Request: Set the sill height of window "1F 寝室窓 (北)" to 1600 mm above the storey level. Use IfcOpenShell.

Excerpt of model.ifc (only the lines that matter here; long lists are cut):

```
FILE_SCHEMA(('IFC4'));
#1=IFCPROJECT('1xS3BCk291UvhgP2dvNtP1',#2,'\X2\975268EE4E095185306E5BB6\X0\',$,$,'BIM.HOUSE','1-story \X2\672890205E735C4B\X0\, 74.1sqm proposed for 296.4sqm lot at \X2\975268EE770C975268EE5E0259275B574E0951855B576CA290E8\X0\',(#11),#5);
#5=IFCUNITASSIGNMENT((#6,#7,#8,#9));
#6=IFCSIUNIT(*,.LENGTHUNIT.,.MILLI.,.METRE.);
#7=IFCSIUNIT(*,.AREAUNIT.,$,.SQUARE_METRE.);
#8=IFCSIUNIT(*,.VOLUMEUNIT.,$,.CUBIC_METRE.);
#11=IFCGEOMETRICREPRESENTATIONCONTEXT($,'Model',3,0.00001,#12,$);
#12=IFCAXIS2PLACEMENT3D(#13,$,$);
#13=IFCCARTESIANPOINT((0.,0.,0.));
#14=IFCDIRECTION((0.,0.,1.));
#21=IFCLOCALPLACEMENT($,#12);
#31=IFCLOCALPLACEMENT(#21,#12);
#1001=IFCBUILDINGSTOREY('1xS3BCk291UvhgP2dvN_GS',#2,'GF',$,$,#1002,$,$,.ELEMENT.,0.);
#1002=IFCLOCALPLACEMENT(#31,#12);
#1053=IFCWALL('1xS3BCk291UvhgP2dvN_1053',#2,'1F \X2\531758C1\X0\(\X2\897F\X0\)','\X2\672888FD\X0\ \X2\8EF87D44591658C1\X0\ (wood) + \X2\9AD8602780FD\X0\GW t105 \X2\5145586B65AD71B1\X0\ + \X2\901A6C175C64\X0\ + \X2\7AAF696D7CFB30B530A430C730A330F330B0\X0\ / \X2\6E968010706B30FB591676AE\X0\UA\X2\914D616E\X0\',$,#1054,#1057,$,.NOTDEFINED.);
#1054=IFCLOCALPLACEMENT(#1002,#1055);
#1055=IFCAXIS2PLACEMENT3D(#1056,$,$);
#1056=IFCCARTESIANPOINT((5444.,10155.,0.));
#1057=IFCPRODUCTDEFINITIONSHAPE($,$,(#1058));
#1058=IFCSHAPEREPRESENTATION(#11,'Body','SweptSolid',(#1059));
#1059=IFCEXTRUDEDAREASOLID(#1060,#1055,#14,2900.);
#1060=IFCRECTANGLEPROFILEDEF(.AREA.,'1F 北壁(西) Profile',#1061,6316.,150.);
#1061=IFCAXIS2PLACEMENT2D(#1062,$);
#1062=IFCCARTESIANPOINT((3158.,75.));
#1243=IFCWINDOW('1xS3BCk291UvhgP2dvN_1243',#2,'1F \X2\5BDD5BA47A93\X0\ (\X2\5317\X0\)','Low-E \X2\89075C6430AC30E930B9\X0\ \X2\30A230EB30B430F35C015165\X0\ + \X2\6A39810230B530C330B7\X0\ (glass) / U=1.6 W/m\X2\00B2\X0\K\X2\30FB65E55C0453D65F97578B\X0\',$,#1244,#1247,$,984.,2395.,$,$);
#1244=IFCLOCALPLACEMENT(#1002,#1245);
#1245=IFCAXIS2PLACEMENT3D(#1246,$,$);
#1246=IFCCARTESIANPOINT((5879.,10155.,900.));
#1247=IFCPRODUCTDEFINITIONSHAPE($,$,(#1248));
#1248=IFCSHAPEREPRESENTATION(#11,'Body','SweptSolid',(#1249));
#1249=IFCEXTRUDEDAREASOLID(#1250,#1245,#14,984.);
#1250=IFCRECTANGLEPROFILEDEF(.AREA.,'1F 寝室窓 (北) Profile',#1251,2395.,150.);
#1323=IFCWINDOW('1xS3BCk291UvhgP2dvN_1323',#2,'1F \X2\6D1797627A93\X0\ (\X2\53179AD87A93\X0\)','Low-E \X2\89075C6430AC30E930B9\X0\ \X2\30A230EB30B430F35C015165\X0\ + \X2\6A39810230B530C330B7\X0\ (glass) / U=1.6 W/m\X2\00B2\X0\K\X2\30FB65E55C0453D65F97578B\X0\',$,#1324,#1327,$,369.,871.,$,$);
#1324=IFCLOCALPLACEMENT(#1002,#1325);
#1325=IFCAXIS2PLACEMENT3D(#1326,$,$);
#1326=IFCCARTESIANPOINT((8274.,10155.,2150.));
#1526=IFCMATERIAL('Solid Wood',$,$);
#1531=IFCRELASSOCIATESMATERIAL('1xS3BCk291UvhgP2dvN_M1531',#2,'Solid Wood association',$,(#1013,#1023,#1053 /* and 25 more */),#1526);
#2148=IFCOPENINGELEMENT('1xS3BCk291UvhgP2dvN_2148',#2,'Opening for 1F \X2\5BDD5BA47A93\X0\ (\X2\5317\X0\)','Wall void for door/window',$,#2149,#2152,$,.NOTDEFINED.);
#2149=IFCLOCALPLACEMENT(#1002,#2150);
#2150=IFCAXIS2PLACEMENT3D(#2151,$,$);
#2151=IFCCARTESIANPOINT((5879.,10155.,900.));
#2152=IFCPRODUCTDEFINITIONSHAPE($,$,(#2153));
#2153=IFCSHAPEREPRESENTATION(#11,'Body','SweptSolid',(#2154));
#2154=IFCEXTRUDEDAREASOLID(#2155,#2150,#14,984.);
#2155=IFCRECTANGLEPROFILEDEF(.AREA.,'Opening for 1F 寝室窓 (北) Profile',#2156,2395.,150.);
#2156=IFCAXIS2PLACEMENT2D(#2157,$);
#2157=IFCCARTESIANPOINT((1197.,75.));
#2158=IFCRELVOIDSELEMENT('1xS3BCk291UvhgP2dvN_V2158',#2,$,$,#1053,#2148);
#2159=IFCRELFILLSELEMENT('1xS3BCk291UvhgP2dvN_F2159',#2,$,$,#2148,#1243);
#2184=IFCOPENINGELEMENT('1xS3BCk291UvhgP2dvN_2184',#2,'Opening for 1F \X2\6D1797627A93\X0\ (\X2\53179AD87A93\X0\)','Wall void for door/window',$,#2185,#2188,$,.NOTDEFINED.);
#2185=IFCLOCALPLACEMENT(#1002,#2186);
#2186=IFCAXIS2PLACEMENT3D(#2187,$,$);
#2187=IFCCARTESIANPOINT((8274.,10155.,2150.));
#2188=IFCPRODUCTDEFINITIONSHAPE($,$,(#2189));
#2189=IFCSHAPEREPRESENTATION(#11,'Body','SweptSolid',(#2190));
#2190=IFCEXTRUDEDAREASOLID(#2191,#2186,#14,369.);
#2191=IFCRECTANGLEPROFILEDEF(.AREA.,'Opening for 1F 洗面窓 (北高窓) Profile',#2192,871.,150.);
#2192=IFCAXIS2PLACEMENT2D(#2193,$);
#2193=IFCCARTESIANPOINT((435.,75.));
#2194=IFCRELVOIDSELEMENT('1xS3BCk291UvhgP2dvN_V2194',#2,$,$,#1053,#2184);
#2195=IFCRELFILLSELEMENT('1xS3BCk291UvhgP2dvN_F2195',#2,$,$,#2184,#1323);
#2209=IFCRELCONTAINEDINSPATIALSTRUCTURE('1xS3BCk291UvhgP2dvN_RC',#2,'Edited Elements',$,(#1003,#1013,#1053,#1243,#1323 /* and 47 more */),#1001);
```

```python
import numpy as np
import ifcopenshell
import ifcopenshell.api.geometry
import ifcopenshell.geom
import ifcopenshell.util.element
import ifcopenshell.util.placement
import ifcopenshell.util.shape
import ifcopenshell.util.unit

model = ifcopenshell.open("model.ifc")
unit_scale = ifcopenshell.util.unit.calculate_unit_scale(model)

window = model.by_guid("1xS3BCk291UvhgP2dvN_1243")
opening = window.FillsVoids[0].RelatingOpeningElement
storey = ifcopenshell.util.element.get_container(window, ifc_class="IfcBuildingStorey")
level = ifcopenshell.util.placement.get_local_placement(storey.ObjectPlacement)[2, 3]

# The opening's origin need not be at the sill, so measure its lowest point.
shape = ifcopenshell.geom.create_shape(ifcopenshell.geom.settings(), opening)
bottom = ifcopenshell.util.shape.get_shape_bottom_elevation(shape, shape.geometry) / unit_scale
dz = level + 1600.0 - bottom

shift = np.array([0.0, 0.0, dz])
# The window is not placed relative to its opening, so move both.
for product in (opening, window):
    matrix = ifcopenshell.util.placement.get_local_placement(product.ObjectPlacement)
    matrix[:3, 3] += shift
    ifcopenshell.api.geometry.edit_object_placement(model, product=product, matrix=matrix, is_si=False)

print(f"moved by {dz * unit_scale:+.3f} m")

model.write("model_rev.ifc")
```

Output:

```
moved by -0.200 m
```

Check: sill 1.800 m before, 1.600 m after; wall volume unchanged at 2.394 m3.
